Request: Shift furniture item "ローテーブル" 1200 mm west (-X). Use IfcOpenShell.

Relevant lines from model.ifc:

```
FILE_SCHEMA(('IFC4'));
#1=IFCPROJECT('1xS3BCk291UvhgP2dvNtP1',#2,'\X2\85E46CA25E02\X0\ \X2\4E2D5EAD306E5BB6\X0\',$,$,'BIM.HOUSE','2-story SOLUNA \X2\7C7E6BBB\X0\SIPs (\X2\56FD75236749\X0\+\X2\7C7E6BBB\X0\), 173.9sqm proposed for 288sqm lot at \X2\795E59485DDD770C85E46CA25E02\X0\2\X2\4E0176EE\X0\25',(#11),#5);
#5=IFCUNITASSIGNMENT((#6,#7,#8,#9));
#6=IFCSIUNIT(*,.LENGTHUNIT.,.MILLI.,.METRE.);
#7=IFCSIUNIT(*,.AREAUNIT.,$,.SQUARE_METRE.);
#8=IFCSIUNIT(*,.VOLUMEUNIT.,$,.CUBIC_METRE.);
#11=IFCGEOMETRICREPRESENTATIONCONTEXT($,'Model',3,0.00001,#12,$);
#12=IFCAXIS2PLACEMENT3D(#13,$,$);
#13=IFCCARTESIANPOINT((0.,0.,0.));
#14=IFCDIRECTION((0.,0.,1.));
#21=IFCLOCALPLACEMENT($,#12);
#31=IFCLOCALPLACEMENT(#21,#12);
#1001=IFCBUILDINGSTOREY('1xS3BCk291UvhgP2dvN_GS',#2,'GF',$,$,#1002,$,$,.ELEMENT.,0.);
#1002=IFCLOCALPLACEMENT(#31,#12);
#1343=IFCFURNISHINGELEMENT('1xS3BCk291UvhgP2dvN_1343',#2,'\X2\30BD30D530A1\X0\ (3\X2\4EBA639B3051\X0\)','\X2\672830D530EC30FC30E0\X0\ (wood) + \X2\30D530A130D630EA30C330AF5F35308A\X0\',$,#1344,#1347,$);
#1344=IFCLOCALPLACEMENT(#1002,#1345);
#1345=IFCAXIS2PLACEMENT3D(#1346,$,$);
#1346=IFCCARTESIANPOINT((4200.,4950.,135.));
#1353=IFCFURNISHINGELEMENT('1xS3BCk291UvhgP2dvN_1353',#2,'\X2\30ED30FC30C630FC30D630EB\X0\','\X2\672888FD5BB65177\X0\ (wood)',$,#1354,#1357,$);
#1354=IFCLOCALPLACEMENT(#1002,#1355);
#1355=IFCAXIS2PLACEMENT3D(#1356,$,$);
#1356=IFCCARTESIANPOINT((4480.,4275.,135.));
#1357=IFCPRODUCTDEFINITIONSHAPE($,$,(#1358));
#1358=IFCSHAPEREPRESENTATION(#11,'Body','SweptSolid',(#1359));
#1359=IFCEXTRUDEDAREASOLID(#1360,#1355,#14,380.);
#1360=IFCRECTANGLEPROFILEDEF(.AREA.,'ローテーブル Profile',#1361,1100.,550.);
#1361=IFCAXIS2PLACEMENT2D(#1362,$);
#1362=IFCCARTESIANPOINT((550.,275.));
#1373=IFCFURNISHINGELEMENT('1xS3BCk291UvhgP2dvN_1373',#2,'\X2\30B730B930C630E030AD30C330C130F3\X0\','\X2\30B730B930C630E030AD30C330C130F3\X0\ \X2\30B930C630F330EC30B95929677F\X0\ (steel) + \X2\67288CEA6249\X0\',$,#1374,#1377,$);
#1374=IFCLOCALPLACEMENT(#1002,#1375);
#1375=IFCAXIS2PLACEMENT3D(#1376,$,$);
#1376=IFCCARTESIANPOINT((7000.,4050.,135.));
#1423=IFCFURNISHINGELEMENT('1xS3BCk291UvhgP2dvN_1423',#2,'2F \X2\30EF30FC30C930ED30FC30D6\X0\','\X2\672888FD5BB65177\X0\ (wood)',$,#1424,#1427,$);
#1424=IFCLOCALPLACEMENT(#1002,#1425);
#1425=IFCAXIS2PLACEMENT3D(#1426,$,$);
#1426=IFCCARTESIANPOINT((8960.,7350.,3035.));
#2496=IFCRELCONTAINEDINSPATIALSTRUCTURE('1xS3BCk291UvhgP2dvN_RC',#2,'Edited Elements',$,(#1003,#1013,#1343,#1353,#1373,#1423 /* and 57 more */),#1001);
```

```python
import ifcopenshell
import ifcopenshell.api.geometry
import ifcopenshell.util.placement
import ifcopenshell.util.unit

model = ifcopenshell.open("model.ifc")
unit_scale = ifcopenshell.util.unit.calculate_unit_scale(model)

item = model.by_guid("1xS3BCk291UvhgP2dvN_1353")
matrix = ifcopenshell.util.placement.get_local_placement(item.ObjectPlacement)
matrix[0, 3] -= 1.2 / unit_scale
ifcopenshell.api.geometry.edit_object_placement(model, product=item, matrix=matrix, is_si=False)

print(ifcopenshell.util.placement.get_local_placement(item.ObjectPlacement).round(3) + 0.0)

model.write("model-out.ifc")
```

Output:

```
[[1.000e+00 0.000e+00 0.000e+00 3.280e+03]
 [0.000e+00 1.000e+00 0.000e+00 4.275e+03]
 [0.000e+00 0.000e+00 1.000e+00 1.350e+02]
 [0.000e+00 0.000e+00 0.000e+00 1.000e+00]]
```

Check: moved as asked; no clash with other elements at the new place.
